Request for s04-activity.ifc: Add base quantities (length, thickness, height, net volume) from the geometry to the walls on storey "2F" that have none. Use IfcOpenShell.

First a look at what the model holds.

```python
import ifcopenshell
import ifcopenshell.util.element
import ifcopenshell.util.unit

model = ifcopenshell.open("s04-activity.ifc")
print(model.schema)
for unit_type in ("LENGTHUNIT", "AREAUNIT", "VOLUMEUNIT"):
    print(unit_type, ifcopenshell.util.unit.calculate_unit_scale(model, unit_type))
storey = next(s for s in model.by_type("IfcBuildingStorey") if s.Name == "2F")
walls = [e for e in ifcopenshell.util.element.get_decomposition(storey) if e.is_a("IfcWall")]
for e in sorted(walls, key=lambda e: e.id()):
    print(e.id(), e.is_a(), e.Name, list(ifcopenshell.util.element.get_psets(e, qtos_only=True)), sep=" | ")
```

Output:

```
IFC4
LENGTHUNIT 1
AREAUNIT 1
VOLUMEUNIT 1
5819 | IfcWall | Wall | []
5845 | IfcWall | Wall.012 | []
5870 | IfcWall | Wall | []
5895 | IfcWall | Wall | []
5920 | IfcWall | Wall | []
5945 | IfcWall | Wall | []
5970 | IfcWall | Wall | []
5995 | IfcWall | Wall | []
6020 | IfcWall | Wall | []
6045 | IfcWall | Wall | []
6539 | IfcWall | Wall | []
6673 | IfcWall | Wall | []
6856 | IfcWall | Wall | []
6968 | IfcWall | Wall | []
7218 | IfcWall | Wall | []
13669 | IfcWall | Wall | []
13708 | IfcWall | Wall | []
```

```python
import ifcopenshell
import ifcopenshell.api.pset
import ifcopenshell.geom
import ifcopenshell.util.element
import ifcopenshell.util.shape
import ifcopenshell.util.unit

model = ifcopenshell.open("s04-activity.ifc")
unit_scale = ifcopenshell.util.unit.calculate_unit_scale(model)
volume_scale = ifcopenshell.util.unit.calculate_unit_scale(model, "VOLUMEUNIT")
settings = ifcopenshell.geom.settings()

storey = next(s for s in model.by_type("IfcBuildingStorey") if s.Name == "2F")
walls = [e for e in ifcopenshell.util.element.get_decomposition(storey) if e.is_a("IfcWall")]

for e in sorted(walls, key=lambda e: e.id()):
    if ifcopenshell.util.element.get_psets(e, qtos_only=True, should_inherit=False):
        continue
    # Geometry comes back in metres, in the element's own axes.
    shape = ifcopenshell.geom.create_shape(settings, e)
    values = {
        "Length": ifcopenshell.util.shape.get_x(shape.geometry) / unit_scale,
        "Width": ifcopenshell.util.shape.get_y(shape.geometry) / unit_scale,
        "Height": ifcopenshell.util.shape.get_z(shape.geometry) / unit_scale,
        "NetVolume": ifcopenshell.util.shape.get_volume(shape.geometry) / volume_scale,
    }
    qto = ifcopenshell.api.pset.add_qto(model, product=e, name="Qto_WallBaseQuantities")
    ifcopenshell.api.pset.edit_qto(model, qto=qto, properties=values)
    print(e.id(), {k: round(v, 3) for k, v in values.items()})

model.write("s04-activity_edited.ifc")
```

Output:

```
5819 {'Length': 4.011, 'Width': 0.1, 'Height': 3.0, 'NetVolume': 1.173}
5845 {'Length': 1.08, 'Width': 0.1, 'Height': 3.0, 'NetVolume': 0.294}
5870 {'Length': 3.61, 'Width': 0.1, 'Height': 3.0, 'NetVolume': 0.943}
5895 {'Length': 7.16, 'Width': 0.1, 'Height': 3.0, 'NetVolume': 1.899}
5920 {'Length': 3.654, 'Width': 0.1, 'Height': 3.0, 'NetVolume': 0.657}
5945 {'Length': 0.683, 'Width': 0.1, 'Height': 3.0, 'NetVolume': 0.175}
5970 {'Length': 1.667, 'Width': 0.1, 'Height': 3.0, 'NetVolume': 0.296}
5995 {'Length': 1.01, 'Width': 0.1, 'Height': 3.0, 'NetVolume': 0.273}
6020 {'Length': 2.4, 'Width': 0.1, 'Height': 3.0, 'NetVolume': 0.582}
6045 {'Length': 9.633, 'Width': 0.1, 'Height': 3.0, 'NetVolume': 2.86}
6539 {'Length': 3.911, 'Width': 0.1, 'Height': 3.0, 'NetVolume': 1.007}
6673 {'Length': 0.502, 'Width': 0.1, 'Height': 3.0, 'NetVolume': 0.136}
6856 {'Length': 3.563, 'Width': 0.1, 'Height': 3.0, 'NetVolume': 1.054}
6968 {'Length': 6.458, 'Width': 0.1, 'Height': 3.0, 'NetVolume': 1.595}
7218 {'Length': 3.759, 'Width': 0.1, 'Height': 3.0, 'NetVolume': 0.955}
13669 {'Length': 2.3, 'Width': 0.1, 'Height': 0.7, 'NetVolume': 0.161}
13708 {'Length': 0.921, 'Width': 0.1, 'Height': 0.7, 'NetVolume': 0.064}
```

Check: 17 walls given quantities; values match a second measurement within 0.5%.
